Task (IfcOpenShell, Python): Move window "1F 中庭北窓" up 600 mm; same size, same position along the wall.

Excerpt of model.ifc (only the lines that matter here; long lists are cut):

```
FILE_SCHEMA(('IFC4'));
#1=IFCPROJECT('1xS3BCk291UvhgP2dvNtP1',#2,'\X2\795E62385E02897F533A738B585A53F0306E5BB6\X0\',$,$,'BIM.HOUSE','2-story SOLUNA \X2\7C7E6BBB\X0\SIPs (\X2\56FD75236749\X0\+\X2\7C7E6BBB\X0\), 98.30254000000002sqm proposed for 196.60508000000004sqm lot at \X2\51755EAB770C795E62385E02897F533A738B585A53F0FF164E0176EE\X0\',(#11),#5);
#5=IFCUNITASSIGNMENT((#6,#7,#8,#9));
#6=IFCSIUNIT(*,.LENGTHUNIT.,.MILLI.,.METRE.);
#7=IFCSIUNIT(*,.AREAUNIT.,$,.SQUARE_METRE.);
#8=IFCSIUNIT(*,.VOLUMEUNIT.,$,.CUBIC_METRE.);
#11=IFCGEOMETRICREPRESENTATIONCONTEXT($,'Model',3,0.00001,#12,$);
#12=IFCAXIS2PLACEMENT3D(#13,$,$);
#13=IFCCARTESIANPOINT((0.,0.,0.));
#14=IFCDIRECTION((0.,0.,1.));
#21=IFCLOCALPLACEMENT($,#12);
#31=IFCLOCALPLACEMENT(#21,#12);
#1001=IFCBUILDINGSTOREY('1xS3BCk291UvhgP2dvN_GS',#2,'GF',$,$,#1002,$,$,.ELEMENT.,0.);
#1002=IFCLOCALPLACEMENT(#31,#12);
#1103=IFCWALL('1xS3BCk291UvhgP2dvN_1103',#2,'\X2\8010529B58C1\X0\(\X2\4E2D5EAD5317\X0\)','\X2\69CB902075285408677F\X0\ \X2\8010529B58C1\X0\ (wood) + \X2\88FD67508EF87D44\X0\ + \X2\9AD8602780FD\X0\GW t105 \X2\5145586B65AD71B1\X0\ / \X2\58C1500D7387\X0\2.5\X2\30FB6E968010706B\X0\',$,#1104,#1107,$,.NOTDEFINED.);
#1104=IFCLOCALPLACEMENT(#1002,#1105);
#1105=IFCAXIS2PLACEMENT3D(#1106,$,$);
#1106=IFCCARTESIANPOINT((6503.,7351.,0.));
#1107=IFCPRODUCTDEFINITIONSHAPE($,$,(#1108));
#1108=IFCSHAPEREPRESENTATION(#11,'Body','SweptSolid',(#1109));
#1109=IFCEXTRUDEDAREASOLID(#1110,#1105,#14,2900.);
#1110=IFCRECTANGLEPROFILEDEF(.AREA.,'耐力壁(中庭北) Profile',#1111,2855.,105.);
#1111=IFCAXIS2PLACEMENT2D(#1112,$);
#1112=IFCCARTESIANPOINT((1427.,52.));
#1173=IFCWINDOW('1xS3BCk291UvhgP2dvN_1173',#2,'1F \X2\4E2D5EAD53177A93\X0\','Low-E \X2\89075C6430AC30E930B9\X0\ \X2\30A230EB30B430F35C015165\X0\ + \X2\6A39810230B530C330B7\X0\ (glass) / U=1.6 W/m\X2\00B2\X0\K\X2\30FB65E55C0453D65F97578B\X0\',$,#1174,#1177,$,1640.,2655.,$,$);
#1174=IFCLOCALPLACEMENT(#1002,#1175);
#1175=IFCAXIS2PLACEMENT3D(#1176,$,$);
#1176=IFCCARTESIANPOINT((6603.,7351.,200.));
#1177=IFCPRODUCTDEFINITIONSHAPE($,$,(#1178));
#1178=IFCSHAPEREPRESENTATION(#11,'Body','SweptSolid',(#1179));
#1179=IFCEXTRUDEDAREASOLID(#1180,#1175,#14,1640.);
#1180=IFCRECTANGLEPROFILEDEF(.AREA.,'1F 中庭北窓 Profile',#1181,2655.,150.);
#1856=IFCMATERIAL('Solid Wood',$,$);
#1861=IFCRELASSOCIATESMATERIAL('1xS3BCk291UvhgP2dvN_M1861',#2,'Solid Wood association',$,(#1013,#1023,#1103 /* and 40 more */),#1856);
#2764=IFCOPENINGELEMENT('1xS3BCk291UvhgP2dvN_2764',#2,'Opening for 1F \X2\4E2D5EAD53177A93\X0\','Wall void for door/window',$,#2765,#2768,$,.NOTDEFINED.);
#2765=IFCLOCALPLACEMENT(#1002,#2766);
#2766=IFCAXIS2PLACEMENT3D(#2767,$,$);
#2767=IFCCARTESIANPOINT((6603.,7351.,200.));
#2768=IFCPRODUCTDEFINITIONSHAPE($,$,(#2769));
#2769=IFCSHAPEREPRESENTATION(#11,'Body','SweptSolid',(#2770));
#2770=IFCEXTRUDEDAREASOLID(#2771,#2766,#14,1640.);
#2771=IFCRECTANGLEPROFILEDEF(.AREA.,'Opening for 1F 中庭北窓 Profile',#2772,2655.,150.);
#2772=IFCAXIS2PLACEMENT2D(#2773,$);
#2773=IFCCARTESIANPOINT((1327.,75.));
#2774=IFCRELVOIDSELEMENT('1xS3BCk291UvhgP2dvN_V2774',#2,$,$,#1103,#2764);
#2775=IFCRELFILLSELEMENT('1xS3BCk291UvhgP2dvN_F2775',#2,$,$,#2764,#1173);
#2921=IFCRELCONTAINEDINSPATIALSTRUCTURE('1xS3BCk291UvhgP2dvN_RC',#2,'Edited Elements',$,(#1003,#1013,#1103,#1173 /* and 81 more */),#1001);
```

```python
import numpy as np
import ifcopenshell
import ifcopenshell.api.geometry
import ifcopenshell.util.placement
import ifcopenshell.util.unit

model = ifcopenshell.open("model.ifc")
unit_scale = ifcopenshell.util.unit.calculate_unit_scale(model)

window = model.by_guid("1xS3BCk291UvhgP2dvN_1173")
opening = window.FillsVoids[0].RelatingOpeningElement
dz = 0.6 / unit_scale

shift = np.array([0.0, 0.0, dz])
# The window is not placed relative to its opening, so move both.
for product in (opening, window):
    matrix = ifcopenshell.util.placement.get_local_placement(product.ObjectPlacement)
    matrix[:3, 3] += shift
    ifcopenshell.api.geometry.edit_object_placement(model, product=product, matrix=matrix, is_si=False)

print(f"moved by {dz * unit_scale:+.3f} m")

model.write("model_updated.ifc")
```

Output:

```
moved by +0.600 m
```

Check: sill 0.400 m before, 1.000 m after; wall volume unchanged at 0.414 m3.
